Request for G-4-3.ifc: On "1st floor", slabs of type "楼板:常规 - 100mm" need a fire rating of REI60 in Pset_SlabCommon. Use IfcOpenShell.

First a look at what the model holds.

```python
import ifcopenshell
import ifcopenshell.util.element

model = ifcopenshell.open("G-4-3.ifc")
print(model.schema)
storey = next(s for s in model.by_type("IfcBuildingStorey") if s.Name == "1st floor")
slabs = [e for e in ifcopenshell.util.element.get_decomposition(storey) if e.is_a("IfcSlab")]
seen = {}
for e in slabs:
    element_type = ifcopenshell.util.element.get_type(e)
    key = (element_type.Name if element_type != e and element_type else None, ifcopenshell.util.element.get_pset(e, "Pset_SlabCommon", "FireRating"))
    seen[key] = seen.get(key, 0) + 1
for (name, value), count in sorted(seen.items(), key=str):
    print(count, "x", name, "|", value)
```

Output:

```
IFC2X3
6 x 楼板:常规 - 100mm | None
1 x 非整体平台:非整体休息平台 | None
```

```python
import ifcopenshell
import ifcopenshell.api.pset
import ifcopenshell.util.element

model = ifcopenshell.open("G-4-3.ifc")

storey = next(s for s in model.by_type("IfcBuildingStorey") if s.Name == "1st floor")
slabs = [e for e in ifcopenshell.util.element.get_decomposition(storey) if e.is_a("IfcSlab")]

count = 0
for e in slabs:
    element_type = ifcopenshell.util.element.get_type(e)
    if element_type in (None, e) or element_type.Name != "楼板:常规 - 100mm":
        continue
    # add_pset returns the element's existing set when there is one.
    pset = ifcopenshell.api.pset.add_pset(model, product=e, name="Pset_SlabCommon")
    ifcopenshell.api.pset.edit_pset(model, pset=pset, properties={"FireRating": "REI60"})
    count += 1

print(count, "slabs updated")

model.write("G-4-3_v2.ifc")
```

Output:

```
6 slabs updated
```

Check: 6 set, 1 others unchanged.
